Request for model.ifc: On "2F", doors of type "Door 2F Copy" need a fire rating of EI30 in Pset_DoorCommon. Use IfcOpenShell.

First a look at what the model holds.

```python
import ifcopenshell
import ifcopenshell.util.element

model = ifcopenshell.open("model.ifc")
print(model.schema)
storey = next(s for s in model.by_type("IfcBuildingStorey") if s.Name == "2F")
doors = [e for e in ifcopenshell.util.element.get_decomposition(storey) if e.is_a("IfcDoor")]
seen = {}
for e in doors:
    element_type = ifcopenshell.util.element.get_type(e)
    key = (element_type.Name if element_type != e and element_type else None, ifcopenshell.util.element.get_pset(e, "Pset_DoorCommon", "FireRating"))
    seen[key] = seen.get(key, 0) + 1
for (name, value), count in sorted(seen.items(), key=str):
    print(count, "x", name, "|", value)
```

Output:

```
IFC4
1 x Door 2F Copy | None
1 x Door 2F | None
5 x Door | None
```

```python
import ifcopenshell
import ifcopenshell.api.pset
import ifcopenshell.util.element

model = ifcopenshell.open("model.ifc")

storey = next(s for s in model.by_type("IfcBuildingStorey") if s.Name == "2F")
doors = [e for e in ifcopenshell.util.element.get_decomposition(storey) if e.is_a("IfcDoor")]

count = 0
for e in doors:
    element_type = ifcopenshell.util.element.get_type(e)
    if element_type in (None, e) or element_type.Name != "Door 2F Copy":
        continue
    # add_pset returns the element's existing set when there is one.
    pset = ifcopenshell.api.pset.add_pset(model, product=e, name="Pset_DoorCommon")
    ifcopenshell.api.pset.edit_pset(model, pset=pset, properties={"FireRating": "EI30"})
    count += 1

print(count, "doors updated")

model.write("model_rev.ifc")
```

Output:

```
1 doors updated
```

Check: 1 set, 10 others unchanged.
